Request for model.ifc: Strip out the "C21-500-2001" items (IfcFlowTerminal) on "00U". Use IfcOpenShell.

First a look at what the model holds.

```python
import ifcopenshell
import ifcopenshell.util.element

model = ifcopenshell.open("model.ifc")
print(model.schema)
storey = next(s for s in model.by_type("IfcBuildingStorey") if s.Name == "00U")
terminals = [e for e in ifcopenshell.util.element.get_decomposition(storey) if e.is_a("IfcFlowTerminal")]
seen = {}
for e in terminals:
    element_type = ifcopenshell.util.element.get_type(e)
    name = element_type.Name if element_type not in (None, e) else None
    seen[name] = seen.get(name, 0) + 1
for name, count in sorted(seen.items(), key=str):
    print(count, "x", name)
```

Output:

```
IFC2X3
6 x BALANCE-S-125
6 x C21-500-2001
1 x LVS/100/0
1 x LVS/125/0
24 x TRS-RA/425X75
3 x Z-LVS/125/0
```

```python
import ifcopenshell
import ifcopenshell.api.root
import ifcopenshell.util.element

model = ifcopenshell.open("model.ifc")

storey = next(s for s in model.by_type("IfcBuildingStorey") if s.Name == "00U")
terminals = [e for e in ifcopenshell.util.element.get_decomposition(storey) if e.is_a("IfcFlowTerminal")]
targets = [e for e in terminals if (t := ifcopenshell.util.element.get_type(e)) not in (None, e) and t.Name == "C21-500-2001"]

for e in targets:
    ifcopenshell.api.root.remove_product(model, product=e)
print(len(targets), "removed")

model.write("model_updated.ifc")
```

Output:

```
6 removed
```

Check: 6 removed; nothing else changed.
